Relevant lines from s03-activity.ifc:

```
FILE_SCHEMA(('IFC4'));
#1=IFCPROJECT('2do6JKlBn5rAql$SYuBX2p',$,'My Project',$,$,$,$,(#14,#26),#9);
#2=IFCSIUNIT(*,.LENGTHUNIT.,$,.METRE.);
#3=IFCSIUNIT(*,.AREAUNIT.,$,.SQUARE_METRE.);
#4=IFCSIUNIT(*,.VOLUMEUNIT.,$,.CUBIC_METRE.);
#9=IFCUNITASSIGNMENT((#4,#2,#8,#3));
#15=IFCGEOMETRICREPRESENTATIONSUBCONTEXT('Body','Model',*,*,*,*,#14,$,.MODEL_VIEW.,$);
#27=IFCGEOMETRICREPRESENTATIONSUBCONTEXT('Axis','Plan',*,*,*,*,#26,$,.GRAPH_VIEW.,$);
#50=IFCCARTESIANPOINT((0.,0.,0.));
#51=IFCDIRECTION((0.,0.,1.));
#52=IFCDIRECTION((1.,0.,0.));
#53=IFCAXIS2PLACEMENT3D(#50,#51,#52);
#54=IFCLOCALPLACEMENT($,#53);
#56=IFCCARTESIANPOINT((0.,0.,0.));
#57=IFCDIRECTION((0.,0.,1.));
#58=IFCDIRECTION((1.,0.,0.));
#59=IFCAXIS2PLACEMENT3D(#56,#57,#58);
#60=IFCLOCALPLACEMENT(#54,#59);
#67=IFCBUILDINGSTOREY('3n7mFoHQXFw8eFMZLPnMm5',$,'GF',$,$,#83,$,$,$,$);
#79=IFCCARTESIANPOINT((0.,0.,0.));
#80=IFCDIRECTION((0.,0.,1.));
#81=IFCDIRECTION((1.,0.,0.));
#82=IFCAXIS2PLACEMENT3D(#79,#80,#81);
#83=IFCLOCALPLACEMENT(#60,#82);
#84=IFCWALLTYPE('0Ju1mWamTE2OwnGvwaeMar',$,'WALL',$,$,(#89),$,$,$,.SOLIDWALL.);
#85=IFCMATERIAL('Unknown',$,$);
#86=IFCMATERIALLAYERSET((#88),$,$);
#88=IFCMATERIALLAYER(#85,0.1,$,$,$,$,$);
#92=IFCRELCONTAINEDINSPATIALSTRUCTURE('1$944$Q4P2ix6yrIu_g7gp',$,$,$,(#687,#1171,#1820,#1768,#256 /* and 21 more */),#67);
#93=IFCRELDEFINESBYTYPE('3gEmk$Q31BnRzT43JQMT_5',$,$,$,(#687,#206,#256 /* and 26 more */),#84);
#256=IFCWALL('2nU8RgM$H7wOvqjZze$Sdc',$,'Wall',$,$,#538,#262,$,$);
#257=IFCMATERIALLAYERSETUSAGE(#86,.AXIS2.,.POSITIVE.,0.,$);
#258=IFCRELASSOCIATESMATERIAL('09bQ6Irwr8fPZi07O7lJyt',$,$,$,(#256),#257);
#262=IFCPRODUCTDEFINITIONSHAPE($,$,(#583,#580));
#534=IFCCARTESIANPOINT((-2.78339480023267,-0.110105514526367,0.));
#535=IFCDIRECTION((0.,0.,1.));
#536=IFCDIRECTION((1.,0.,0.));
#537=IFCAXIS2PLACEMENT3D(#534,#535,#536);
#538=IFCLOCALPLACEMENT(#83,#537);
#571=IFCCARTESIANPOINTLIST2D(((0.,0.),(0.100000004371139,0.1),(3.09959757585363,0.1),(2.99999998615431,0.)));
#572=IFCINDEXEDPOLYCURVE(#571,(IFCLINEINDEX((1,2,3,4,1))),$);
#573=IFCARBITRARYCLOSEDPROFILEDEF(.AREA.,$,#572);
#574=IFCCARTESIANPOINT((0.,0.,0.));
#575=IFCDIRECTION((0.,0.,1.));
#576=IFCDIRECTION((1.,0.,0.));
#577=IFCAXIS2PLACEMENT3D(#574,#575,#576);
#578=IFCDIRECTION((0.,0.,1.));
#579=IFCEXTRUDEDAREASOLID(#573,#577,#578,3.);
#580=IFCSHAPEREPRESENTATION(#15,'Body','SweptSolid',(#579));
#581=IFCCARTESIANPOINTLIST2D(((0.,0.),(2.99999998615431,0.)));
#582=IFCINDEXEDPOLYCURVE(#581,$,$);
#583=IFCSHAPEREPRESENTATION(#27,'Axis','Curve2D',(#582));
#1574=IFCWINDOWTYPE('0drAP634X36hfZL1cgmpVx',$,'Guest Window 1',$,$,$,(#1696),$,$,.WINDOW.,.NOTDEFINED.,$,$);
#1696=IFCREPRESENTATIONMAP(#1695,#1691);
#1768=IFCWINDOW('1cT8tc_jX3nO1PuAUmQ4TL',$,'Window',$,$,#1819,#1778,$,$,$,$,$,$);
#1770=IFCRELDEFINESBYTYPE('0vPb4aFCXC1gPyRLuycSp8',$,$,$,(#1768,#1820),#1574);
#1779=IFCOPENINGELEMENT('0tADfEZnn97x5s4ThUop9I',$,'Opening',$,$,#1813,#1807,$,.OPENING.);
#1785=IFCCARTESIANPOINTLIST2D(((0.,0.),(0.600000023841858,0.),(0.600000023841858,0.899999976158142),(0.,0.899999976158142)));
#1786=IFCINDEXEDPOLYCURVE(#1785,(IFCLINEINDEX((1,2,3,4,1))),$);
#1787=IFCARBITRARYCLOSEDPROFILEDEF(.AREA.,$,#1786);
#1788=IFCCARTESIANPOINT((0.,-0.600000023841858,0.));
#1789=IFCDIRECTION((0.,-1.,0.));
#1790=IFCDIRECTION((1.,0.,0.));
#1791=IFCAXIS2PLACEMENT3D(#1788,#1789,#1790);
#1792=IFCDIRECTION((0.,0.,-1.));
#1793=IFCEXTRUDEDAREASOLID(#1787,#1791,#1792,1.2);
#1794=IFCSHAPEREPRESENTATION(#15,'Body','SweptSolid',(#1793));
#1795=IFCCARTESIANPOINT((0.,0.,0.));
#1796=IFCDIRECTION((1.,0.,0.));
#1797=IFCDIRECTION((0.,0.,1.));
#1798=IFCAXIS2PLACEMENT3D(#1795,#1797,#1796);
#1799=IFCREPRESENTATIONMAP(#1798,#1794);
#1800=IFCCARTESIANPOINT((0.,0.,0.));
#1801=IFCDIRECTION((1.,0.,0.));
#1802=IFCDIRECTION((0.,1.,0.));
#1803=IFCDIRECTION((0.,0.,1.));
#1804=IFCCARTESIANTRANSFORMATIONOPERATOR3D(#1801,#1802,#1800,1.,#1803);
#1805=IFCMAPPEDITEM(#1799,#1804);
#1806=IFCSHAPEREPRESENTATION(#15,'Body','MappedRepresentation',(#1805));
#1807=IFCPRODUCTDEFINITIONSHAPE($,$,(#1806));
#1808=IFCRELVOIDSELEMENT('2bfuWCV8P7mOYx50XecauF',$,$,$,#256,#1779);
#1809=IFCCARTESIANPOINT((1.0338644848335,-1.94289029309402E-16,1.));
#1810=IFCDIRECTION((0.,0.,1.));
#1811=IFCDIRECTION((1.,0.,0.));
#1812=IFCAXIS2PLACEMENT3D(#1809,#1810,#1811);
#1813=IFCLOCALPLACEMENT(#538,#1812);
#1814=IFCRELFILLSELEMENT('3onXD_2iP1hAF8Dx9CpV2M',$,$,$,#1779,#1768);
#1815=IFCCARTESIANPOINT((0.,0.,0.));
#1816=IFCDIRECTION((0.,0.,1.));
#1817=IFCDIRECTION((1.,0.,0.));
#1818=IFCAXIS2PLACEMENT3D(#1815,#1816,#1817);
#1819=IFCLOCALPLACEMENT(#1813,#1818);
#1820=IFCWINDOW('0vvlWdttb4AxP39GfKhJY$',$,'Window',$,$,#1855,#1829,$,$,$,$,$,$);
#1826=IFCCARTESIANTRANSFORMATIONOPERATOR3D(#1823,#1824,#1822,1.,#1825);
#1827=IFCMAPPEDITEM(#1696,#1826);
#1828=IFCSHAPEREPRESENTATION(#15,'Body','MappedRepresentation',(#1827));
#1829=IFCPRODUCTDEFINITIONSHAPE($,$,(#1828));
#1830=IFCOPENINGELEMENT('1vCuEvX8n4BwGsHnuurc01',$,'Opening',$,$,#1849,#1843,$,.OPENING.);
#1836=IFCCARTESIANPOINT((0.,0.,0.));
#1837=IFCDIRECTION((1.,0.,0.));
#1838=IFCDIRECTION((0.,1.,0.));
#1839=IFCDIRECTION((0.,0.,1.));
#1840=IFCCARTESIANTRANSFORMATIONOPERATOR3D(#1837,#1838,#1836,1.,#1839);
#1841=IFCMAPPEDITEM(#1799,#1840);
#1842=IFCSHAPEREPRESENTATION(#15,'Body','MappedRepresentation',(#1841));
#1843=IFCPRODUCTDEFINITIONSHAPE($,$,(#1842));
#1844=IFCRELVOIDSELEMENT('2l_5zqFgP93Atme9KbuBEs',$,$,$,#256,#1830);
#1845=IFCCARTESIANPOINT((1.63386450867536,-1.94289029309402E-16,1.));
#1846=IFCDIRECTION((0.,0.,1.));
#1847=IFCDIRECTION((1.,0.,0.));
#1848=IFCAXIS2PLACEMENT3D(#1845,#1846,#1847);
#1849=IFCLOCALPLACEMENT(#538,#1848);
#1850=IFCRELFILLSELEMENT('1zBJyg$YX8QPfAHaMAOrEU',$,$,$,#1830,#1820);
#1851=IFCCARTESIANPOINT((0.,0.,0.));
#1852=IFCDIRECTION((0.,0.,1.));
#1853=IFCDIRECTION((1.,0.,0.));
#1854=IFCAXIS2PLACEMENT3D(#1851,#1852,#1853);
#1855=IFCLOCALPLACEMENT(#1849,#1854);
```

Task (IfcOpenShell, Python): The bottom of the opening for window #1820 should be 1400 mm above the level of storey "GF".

```python
import numpy as np
import ifcopenshell
import ifcopenshell.api.geometry
import ifcopenshell.geom
import ifcopenshell.util.element
import ifcopenshell.util.placement
import ifcopenshell.util.shape
import ifcopenshell.util.unit

model = ifcopenshell.open("s03-activity.ifc")
unit_scale = ifcopenshell.util.unit.calculate_unit_scale(model)

window = model.by_guid("0vvlWdttb4AxP39GfKhJY$")
opening = window.FillsVoids[0].RelatingOpeningElement
storey = ifcopenshell.util.element.get_container(window, ifc_class="IfcBuildingStorey")
level = ifcopenshell.util.placement.get_local_placement(storey.ObjectPlacement)[2, 3]

# The opening's origin need not be at the sill, so measure its lowest point.
shape = ifcopenshell.geom.create_shape(ifcopenshell.geom.settings(), opening)
bottom = ifcopenshell.util.shape.get_shape_bottom_elevation(shape, shape.geometry) / unit_scale
dz = level + 1.4 / unit_scale - bottom

shift = np.array([0.0, 0.0, dz])
# The window is placed relative to its opening, so it follows when the opening moves.
matrix = ifcopenshell.util.placement.get_local_placement(opening.ObjectPlacement)
matrix[:3, 3] += shift
ifcopenshell.api.geometry.edit_object_placement(
    model, product=opening, matrix=matrix, is_si=False, should_transform_children=True
)

print(f"moved by {dz * unit_scale:+.3f} m")

model.write("s03-activity_rev.ifc")
```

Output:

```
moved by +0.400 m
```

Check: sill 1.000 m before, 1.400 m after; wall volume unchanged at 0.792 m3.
